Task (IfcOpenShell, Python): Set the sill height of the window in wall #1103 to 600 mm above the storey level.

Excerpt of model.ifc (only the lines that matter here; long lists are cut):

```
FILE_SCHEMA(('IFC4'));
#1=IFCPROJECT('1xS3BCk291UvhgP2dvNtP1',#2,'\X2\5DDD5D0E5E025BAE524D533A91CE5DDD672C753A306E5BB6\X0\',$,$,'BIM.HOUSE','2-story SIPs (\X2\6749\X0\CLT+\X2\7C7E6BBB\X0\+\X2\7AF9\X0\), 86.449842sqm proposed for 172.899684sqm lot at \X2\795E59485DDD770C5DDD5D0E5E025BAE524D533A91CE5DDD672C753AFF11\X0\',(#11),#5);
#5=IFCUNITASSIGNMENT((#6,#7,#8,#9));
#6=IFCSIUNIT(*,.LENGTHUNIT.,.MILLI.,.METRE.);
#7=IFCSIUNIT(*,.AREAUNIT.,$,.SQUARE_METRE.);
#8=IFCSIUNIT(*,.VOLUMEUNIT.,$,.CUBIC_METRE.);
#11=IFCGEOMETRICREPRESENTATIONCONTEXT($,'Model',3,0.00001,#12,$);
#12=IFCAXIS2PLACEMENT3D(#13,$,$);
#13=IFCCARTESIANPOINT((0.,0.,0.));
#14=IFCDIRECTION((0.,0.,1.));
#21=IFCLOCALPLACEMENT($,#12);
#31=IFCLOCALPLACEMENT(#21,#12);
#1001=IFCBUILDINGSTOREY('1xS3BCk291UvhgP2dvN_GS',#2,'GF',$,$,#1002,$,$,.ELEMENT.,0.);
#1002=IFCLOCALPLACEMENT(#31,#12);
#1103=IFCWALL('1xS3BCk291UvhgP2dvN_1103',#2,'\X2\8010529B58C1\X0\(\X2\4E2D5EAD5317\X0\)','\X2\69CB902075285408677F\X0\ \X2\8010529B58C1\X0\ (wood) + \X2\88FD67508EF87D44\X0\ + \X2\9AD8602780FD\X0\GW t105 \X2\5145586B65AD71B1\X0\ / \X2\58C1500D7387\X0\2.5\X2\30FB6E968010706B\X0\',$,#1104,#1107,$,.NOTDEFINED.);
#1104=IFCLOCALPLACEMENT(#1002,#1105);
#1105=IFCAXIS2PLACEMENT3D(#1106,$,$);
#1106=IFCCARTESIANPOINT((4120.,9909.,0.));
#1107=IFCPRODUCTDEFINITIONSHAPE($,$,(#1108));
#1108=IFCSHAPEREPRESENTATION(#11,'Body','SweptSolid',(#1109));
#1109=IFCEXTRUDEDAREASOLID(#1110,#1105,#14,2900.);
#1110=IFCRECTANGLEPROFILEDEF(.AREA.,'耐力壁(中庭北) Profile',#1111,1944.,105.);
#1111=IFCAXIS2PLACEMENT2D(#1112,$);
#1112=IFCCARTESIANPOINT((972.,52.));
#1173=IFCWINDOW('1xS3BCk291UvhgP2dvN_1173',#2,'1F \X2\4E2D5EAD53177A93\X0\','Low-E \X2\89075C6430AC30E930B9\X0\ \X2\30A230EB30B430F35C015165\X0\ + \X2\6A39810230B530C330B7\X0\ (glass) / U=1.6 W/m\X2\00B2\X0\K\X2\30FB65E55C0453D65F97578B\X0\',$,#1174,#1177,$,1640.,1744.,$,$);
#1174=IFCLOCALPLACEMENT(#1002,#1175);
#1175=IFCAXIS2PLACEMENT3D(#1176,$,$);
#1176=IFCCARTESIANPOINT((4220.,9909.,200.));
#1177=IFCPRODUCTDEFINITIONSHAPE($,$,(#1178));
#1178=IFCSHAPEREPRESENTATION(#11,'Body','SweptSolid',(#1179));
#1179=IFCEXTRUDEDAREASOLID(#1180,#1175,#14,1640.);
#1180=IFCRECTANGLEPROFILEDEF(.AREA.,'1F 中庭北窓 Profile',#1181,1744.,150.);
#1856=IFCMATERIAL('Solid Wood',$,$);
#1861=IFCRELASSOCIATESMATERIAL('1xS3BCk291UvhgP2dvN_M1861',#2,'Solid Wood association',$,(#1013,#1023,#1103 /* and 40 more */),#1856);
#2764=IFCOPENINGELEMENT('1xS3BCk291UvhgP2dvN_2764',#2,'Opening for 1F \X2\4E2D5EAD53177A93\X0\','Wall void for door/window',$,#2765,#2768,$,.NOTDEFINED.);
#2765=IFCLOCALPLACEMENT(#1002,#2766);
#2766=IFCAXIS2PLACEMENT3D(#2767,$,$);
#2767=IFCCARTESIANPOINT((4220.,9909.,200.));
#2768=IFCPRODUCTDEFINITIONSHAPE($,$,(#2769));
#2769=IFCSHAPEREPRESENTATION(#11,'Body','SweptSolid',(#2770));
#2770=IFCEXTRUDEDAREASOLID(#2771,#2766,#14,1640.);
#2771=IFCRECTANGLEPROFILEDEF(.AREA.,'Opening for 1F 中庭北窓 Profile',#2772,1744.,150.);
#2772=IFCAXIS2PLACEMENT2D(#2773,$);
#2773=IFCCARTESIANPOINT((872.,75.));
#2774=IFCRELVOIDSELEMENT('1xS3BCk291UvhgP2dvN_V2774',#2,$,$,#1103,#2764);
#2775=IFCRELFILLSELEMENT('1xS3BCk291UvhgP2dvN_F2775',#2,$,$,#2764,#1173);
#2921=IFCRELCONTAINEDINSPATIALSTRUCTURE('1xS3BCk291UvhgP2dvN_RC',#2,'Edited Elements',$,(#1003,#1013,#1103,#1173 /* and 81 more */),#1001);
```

```python
import numpy as np
import ifcopenshell
import ifcopenshell.api.geometry
import ifcopenshell.geom
import ifcopenshell.util.element
import ifcopenshell.util.placement
import ifcopenshell.util.shape
import ifcopenshell.util.unit

model = ifcopenshell.open("model.ifc")
unit_scale = ifcopenshell.util.unit.calculate_unit_scale(model)

window = model.by_id(1173)
opening = window.FillsVoids[0].RelatingOpeningElement
storey = ifcopenshell.util.element.get_container(window, ifc_class="IfcBuildingStorey")
level = ifcopenshell.util.placement.get_local_placement(storey.ObjectPlacement)[2, 3]

# The opening's origin need not be at the sill, so measure its lowest point.
shape = ifcopenshell.geom.create_shape(ifcopenshell.geom.settings(), opening)
bottom = ifcopenshell.util.shape.get_shape_bottom_elevation(shape, shape.geometry) / unit_scale
dz = level + 0.6 / unit_scale - bottom

shift = np.array([0.0, 0.0, dz])
# The window is not placed relative to its opening, so move both.
for product in (opening, window):
    matrix = ifcopenshell.util.placement.get_local_placement(product.ObjectPlacement)
    matrix[:3, 3] += shift
    ifcopenshell.api.geometry.edit_object_placement(model, product=product, matrix=matrix, is_si=False)

print(f"moved by {dz * unit_scale:+.3f} m")

model.write("model_v2.ifc")
```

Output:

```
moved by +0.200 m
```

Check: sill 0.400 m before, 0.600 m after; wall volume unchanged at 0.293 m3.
